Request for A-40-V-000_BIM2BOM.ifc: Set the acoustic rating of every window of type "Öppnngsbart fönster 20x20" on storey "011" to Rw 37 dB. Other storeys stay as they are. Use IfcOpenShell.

First a look at what the model holds.

```python
import ifcopenshell
import ifcopenshell.util.element

model = ifcopenshell.open("A-40-V-000_BIM2BOM.ifc")
print(model.schema)
storey = next(s for s in model.by_type("IfcBuildingStorey") if s.Name == "011")
windows = [e for e in ifcopenshell.util.element.get_decomposition(storey) if e.is_a("IfcWindow")]
seen = {}
for e in windows:
    element_type = ifcopenshell.util.element.get_type(e)
    key = (element_type.Name if element_type != e and element_type else None, ifcopenshell.util.element.get_pset(e, "Pset_WindowCommon", "AcousticRating"))
    seen[key] = seen.get(key, 0) + 1
for (name, value), count in sorted(seen.items(), key=str):
    print(count, "x", name, "|", value)
```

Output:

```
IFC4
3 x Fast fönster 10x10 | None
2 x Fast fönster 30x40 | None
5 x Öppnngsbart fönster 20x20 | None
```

```python
import ifcopenshell
import ifcopenshell.api.pset
import ifcopenshell.util.element

model = ifcopenshell.open("A-40-V-000_BIM2BOM.ifc")

storey = next(s for s in model.by_type("IfcBuildingStorey") if s.Name == "011")
windows = [e for e in ifcopenshell.util.element.get_decomposition(storey) if e.is_a("IfcWindow")]

count = 0
for e in windows:
    element_type = ifcopenshell.util.element.get_type(e)
    if element_type in (None, e) or element_type.Name != "Öppnngsbart fönster 20x20":
        continue
    # add_pset returns the element's existing set when there is one.
    pset = ifcopenshell.api.pset.add_pset(model, product=e, name="Pset_WindowCommon")
    ifcopenshell.api.pset.edit_pset(model, pset=pset, properties={"AcousticRating": "Rw 37 dB"})
    count += 1

print(count, "windows updated")

model.write("A-40-V-000_BIM2BOM-out.ifc")
```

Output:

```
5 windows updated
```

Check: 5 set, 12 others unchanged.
